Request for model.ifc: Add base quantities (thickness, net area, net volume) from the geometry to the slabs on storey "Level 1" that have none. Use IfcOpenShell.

First a look at what the model holds.

```python
import ifcopenshell
import ifcopenshell.util.element
import ifcopenshell.util.unit

model = ifcopenshell.open("model.ifc")
print(model.schema)
for unit_type in ("LENGTHUNIT", "AREAUNIT", "VOLUMEUNIT"):
    print(unit_type, ifcopenshell.util.unit.calculate_unit_scale(model, unit_type))
storey = next(s for s in model.by_type("IfcBuildingStorey") if s.Name == "Level 1")
slabs = [e for e in ifcopenshell.util.element.get_decomposition(storey) if e.is_a("IfcSlab")]
for e in sorted(slabs, key=lambda e: e.id()):
    print(e.id(), e.is_a(), e.Name, list(ifcopenshell.util.element.get_psets(e, qtos_only=True)), sep=" | ")
```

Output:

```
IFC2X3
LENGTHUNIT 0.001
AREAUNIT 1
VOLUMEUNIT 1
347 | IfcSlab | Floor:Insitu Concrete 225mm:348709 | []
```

```python
import ifcopenshell
import ifcopenshell.api.pset
import ifcopenshell.geom
import ifcopenshell.util.element
import ifcopenshell.util.shape
import ifcopenshell.util.unit

model = ifcopenshell.open("model.ifc")
unit_scale = ifcopenshell.util.unit.calculate_unit_scale(model)
area_scale = ifcopenshell.util.unit.calculate_unit_scale(model, "AREAUNIT")
volume_scale = ifcopenshell.util.unit.calculate_unit_scale(model, "VOLUMEUNIT")
settings = ifcopenshell.geom.settings()

storey = next(s for s in model.by_type("IfcBuildingStorey") if s.Name == "Level 1")
slabs = [e for e in ifcopenshell.util.element.get_decomposition(storey) if e.is_a("IfcSlab")]

for e in sorted(slabs, key=lambda e: e.id()):
    if ifcopenshell.util.element.get_psets(e, qtos_only=True, should_inherit=False):
        continue
    # Geometry comes back in metres, in the element's own axes.
    shape = ifcopenshell.geom.create_shape(settings, e)
    values = {
        "Width": ifcopenshell.util.shape.get_z(shape.geometry) / unit_scale,
        "NetArea": ifcopenshell.util.shape.get_footprint_area(shape.geometry) / area_scale,
        "NetVolume": ifcopenshell.util.shape.get_volume(shape.geometry) / volume_scale,
    }
    qto = ifcopenshell.api.pset.add_qto(model, product=e, name="BaseQuantities")
    ifcopenshell.api.pset.edit_qto(model, qto=qto, properties=values)
    print(e.id(), {k: round(v, 3) for k, v in values.items()})

model.write("model_edited.ifc")
```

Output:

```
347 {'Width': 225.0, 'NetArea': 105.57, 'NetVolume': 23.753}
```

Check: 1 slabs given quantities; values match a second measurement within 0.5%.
